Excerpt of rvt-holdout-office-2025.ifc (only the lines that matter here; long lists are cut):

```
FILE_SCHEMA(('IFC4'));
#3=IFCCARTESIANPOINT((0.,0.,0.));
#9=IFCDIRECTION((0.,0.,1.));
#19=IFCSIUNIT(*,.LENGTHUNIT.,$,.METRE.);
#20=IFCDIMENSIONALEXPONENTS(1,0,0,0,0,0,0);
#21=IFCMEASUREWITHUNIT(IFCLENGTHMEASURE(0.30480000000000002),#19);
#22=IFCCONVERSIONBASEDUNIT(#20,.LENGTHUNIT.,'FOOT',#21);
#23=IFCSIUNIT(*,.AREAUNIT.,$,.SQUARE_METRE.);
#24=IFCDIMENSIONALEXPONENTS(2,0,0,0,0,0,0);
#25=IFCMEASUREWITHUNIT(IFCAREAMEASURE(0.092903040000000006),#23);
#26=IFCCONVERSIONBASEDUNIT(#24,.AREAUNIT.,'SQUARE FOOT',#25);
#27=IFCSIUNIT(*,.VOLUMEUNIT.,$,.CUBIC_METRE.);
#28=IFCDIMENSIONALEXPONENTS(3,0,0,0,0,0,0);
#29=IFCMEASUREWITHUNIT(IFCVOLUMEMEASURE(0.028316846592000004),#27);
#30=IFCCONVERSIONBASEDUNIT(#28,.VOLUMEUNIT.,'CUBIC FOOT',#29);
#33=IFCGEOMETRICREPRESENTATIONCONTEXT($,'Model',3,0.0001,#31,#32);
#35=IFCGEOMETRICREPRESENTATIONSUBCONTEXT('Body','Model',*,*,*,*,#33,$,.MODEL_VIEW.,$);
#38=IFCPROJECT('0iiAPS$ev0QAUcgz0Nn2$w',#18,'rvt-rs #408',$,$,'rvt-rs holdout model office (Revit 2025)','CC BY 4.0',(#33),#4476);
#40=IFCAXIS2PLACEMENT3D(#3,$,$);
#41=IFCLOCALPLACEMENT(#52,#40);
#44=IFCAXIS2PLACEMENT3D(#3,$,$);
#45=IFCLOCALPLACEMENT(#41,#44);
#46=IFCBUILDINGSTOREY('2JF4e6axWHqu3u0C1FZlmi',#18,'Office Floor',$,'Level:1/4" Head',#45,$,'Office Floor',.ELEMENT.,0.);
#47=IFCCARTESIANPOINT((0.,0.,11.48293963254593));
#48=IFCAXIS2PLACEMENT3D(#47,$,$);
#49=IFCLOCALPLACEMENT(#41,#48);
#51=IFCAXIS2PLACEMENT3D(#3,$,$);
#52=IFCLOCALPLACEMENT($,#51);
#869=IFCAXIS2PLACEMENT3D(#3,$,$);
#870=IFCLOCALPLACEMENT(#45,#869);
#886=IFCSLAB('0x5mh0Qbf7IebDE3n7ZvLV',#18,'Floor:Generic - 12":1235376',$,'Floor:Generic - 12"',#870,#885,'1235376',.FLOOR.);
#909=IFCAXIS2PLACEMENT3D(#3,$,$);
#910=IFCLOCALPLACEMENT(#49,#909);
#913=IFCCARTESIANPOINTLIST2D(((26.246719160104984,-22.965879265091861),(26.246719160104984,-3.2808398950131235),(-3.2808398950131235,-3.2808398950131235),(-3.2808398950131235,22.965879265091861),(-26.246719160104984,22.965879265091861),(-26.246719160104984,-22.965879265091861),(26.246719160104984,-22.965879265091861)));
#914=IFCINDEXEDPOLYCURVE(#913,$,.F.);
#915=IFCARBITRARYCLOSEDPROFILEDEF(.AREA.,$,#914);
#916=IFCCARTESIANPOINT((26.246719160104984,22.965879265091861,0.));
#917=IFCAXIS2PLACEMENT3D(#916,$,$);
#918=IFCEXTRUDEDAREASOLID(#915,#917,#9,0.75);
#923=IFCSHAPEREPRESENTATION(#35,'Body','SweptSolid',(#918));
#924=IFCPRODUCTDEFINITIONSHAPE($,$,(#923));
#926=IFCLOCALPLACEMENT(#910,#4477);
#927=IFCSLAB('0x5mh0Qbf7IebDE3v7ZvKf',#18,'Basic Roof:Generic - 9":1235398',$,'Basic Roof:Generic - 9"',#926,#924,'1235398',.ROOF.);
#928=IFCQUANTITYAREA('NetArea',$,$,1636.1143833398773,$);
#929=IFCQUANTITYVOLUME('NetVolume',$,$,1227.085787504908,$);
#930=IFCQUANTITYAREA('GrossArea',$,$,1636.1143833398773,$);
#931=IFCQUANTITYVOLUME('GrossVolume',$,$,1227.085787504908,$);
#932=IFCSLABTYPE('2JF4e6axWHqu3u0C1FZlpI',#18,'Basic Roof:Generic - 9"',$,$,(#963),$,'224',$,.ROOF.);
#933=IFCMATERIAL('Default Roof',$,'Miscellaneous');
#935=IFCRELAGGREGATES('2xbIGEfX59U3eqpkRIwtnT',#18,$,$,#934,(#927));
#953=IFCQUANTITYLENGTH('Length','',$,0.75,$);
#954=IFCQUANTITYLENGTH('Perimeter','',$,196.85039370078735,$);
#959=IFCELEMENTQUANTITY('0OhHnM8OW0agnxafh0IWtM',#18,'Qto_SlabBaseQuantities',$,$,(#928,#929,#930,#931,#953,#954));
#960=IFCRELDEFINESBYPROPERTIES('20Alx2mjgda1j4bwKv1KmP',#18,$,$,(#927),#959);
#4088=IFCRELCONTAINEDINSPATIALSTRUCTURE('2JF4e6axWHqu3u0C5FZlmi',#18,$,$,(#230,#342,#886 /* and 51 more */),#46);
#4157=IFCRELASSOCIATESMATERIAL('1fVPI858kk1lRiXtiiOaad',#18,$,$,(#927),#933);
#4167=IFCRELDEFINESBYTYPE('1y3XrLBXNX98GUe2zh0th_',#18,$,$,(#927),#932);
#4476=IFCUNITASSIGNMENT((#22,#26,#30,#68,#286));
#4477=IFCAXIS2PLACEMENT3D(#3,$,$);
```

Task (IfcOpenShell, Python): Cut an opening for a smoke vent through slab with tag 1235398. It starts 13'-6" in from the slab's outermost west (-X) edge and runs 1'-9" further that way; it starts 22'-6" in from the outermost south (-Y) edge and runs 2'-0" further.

```python
import numpy as np
import ifcopenshell
import ifcopenshell.api.feature
import ifcopenshell.api.geometry
import ifcopenshell.api.pset
import ifcopenshell.api.root
import ifcopenshell.geom
import ifcopenshell.util.element
import ifcopenshell.util.placement
import ifcopenshell.util.representation
import ifcopenshell.util.shape
import ifcopenshell.util.unit

model = ifcopenshell.open("rvt-holdout-office-2025.ifc")
unit_scale = ifcopenshell.util.unit.calculate_unit_scale(model)
area_scale = ifcopenshell.util.unit.calculate_unit_scale(model, "AREAUNIT")
volume_scale = ifcopenshell.util.unit.calculate_unit_scale(model, "VOLUMEUNIT")
settings = ifcopenshell.geom.settings()


def volume(element):
    """Net volume in cubic metres, openings subtracted."""
    shape = ifcopenshell.geom.create_shape(settings, element)
    return ifcopenshell.util.shape.get_volume(shape.geometry)


slab = model.by_guid("0x5mh0Qbf7IebDE3v7ZvKf")
before = volume(slab)

# Extent in the slab's own axes, in metres. The edges named are its -X and -Y sides.
slab_shape = ifcopenshell.geom.create_shape(settings, slab)
vertices = ifcopenshell.util.shape.get_vertices(slab_shape.geometry)
x_min, y_min, bottom = vertices.min(axis=0)
top = vertices[:, 2].max()

opening = ifcopenshell.api.root.create_entity(model, ifc_class="IfcOpeningElement", name="Smoke vent opening", predefined_type="OPENING")
context = ifcopenshell.util.representation.get_context(model, "Model", "Body", "MODEL_VIEW")
width, depth = 0.5334, 0.6096
outline = [(0.0, 0.0), (width, 0.0), (width, depth), (0.0, depth), (0.0, 0.0)]
# Overshoot both faces by 50 mm so the cut is clean.
shape = ifcopenshell.api.geometry.add_slab_representation(
    model, context=context, depth=top - bottom + 0.1, polyline=outline
)
ifcopenshell.api.geometry.assign_representation(model, product=opening, representation=shape)

matrix = ifcopenshell.util.placement.get_local_placement(slab.ObjectPlacement)
matrix[:, 3] = matrix @ np.append(np.array([x_min + 4.1148, y_min + 6.858, bottom - 0.05]) / unit_scale, 1.0)
ifcopenshell.api.geometry.edit_object_placement(model, product=opening, matrix=matrix, is_si=False)
ifcopenshell.api.feature.add_feature(model, feature=opening, element=slab)

after = volume(slab)

# Update the slab's stored quantities.
qto = model.by_id(ifcopenshell.util.element.get_pset(slab, "Qto_SlabBaseQuantities", should_inherit=False)["id"])
ifcopenshell.api.pset.edit_qto(model, qto=qto, properties={
    "NetArea": after / (top - bottom) / area_scale,
    "NetVolume": after / volume_scale,
})

print(f"slab volume {before:.3f} -> {after:.3f} m3")

model.write("rvt-holdout-office-2025_v2.ifc")
```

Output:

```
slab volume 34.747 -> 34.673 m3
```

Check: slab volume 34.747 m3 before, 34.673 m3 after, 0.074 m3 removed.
